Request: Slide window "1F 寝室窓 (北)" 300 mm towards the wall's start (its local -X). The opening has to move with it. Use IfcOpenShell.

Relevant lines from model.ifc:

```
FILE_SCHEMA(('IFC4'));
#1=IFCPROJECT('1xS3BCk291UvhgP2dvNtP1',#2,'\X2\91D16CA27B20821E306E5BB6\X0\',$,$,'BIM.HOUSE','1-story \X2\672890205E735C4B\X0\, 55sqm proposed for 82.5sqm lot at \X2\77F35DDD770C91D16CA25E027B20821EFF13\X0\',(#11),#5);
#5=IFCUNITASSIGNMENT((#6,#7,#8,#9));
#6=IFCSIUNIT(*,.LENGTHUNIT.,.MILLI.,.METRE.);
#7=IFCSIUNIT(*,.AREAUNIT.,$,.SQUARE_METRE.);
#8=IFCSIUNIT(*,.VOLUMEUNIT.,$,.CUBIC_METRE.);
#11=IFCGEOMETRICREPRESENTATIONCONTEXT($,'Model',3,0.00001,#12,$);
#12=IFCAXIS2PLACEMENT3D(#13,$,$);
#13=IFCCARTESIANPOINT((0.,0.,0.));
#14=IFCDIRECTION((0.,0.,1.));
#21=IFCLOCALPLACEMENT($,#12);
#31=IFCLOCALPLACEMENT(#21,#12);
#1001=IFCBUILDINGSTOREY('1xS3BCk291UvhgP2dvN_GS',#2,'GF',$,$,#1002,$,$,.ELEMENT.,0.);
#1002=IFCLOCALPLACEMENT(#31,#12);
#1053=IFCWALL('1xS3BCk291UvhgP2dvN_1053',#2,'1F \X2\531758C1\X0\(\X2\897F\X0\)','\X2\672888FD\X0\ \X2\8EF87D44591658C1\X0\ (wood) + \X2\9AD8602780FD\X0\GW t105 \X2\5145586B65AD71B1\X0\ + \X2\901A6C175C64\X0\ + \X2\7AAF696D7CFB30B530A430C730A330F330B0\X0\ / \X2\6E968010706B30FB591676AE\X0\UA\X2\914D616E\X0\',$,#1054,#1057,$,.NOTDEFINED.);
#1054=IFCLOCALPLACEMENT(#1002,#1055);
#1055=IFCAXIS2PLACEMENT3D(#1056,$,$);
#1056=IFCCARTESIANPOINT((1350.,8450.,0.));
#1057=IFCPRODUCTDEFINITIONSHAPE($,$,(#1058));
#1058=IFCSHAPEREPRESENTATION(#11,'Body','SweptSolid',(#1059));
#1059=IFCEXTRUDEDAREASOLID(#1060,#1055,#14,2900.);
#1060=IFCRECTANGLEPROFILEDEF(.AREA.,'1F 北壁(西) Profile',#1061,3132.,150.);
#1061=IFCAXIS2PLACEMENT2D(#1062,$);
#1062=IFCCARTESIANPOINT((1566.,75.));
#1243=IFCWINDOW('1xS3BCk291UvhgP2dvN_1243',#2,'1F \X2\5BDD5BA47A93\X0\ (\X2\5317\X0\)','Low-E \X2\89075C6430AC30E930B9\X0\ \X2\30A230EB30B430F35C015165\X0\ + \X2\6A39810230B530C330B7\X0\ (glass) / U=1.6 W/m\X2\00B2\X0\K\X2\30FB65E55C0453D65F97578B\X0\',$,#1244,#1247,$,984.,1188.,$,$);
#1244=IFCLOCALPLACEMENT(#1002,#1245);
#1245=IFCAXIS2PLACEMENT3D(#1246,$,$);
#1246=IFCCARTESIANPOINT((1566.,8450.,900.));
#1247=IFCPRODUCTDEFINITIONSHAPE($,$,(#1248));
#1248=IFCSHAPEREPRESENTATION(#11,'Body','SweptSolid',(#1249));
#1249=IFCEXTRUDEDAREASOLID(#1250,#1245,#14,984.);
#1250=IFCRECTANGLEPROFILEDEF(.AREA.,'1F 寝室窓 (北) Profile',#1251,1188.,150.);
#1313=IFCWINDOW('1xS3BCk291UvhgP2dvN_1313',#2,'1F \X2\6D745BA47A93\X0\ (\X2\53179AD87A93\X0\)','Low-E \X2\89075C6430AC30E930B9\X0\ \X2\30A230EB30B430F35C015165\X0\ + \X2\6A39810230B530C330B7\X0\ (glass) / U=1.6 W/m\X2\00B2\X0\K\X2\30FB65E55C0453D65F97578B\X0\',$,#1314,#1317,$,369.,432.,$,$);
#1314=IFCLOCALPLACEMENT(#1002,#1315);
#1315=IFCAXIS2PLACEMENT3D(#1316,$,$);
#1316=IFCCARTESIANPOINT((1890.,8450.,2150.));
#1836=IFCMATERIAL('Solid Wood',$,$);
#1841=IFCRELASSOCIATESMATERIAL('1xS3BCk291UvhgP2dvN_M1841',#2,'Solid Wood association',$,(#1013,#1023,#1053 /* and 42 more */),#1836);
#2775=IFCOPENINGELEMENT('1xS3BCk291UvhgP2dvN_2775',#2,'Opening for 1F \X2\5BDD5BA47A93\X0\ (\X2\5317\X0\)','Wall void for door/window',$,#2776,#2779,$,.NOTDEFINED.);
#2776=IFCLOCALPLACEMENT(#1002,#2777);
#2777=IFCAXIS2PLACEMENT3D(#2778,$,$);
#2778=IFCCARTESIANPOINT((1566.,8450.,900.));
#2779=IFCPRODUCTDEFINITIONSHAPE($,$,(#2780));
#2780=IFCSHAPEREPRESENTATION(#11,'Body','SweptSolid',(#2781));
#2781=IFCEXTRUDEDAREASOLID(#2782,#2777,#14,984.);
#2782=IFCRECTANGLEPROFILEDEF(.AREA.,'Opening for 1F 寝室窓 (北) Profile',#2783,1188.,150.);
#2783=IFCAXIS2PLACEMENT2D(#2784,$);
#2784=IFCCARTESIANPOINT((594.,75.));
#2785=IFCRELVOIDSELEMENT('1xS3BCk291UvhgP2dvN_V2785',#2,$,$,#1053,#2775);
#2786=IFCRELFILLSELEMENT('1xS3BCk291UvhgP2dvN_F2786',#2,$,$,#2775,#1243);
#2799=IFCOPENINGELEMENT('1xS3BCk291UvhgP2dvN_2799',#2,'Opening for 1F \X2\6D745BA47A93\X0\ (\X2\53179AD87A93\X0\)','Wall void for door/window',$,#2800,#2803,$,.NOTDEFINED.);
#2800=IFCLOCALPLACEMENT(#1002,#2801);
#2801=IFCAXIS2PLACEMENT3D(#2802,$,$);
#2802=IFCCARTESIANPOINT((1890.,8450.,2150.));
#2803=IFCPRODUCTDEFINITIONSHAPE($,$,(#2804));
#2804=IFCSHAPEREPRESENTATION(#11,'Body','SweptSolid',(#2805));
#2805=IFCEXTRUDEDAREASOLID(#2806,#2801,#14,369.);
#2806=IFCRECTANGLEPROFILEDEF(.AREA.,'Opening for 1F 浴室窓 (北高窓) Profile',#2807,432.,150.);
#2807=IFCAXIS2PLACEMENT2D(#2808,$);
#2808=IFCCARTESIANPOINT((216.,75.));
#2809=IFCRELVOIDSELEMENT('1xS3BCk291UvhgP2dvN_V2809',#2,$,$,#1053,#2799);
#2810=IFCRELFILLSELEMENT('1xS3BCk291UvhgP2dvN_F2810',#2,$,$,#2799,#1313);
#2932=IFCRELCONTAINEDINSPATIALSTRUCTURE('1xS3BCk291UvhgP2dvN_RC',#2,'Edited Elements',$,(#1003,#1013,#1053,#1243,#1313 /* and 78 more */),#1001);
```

```python
import ifcopenshell
import ifcopenshell.api.geometry
import ifcopenshell.util.placement
import ifcopenshell.util.unit

model = ifcopenshell.open("model.ifc")
unit_scale = ifcopenshell.util.unit.calculate_unit_scale(model)

window = model.by_guid("1xS3BCk291UvhgP2dvN_1243")
opening = window.FillsVoids[0].RelatingOpeningElement
wall = opening.VoidsElements[0].RelatingBuildingElement

wall_matrix = ifcopenshell.util.placement.get_local_placement(wall.ObjectPlacement)
shift = wall_matrix[:3, 0] * -0.3 / unit_scale
before = ifcopenshell.util.placement.get_local_placement(window.ObjectPlacement)[:3, 3].copy()

# The window is not placed relative to its opening, so move both.
for product in (opening, window):
    matrix = ifcopenshell.util.placement.get_local_placement(product.ObjectPlacement)
    matrix[:3, 3] += shift
    ifcopenshell.api.geometry.edit_object_placement(model, product=product, matrix=matrix, is_si=False)

after = ifcopenshell.util.placement.get_local_placement(window.ObjectPlacement)[:3, 3]
print("window moved by", (after - before).round(3) + 0.0)

model.write("model-out.ifc")
```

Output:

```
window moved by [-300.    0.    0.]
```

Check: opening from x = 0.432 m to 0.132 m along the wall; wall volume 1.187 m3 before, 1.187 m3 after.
